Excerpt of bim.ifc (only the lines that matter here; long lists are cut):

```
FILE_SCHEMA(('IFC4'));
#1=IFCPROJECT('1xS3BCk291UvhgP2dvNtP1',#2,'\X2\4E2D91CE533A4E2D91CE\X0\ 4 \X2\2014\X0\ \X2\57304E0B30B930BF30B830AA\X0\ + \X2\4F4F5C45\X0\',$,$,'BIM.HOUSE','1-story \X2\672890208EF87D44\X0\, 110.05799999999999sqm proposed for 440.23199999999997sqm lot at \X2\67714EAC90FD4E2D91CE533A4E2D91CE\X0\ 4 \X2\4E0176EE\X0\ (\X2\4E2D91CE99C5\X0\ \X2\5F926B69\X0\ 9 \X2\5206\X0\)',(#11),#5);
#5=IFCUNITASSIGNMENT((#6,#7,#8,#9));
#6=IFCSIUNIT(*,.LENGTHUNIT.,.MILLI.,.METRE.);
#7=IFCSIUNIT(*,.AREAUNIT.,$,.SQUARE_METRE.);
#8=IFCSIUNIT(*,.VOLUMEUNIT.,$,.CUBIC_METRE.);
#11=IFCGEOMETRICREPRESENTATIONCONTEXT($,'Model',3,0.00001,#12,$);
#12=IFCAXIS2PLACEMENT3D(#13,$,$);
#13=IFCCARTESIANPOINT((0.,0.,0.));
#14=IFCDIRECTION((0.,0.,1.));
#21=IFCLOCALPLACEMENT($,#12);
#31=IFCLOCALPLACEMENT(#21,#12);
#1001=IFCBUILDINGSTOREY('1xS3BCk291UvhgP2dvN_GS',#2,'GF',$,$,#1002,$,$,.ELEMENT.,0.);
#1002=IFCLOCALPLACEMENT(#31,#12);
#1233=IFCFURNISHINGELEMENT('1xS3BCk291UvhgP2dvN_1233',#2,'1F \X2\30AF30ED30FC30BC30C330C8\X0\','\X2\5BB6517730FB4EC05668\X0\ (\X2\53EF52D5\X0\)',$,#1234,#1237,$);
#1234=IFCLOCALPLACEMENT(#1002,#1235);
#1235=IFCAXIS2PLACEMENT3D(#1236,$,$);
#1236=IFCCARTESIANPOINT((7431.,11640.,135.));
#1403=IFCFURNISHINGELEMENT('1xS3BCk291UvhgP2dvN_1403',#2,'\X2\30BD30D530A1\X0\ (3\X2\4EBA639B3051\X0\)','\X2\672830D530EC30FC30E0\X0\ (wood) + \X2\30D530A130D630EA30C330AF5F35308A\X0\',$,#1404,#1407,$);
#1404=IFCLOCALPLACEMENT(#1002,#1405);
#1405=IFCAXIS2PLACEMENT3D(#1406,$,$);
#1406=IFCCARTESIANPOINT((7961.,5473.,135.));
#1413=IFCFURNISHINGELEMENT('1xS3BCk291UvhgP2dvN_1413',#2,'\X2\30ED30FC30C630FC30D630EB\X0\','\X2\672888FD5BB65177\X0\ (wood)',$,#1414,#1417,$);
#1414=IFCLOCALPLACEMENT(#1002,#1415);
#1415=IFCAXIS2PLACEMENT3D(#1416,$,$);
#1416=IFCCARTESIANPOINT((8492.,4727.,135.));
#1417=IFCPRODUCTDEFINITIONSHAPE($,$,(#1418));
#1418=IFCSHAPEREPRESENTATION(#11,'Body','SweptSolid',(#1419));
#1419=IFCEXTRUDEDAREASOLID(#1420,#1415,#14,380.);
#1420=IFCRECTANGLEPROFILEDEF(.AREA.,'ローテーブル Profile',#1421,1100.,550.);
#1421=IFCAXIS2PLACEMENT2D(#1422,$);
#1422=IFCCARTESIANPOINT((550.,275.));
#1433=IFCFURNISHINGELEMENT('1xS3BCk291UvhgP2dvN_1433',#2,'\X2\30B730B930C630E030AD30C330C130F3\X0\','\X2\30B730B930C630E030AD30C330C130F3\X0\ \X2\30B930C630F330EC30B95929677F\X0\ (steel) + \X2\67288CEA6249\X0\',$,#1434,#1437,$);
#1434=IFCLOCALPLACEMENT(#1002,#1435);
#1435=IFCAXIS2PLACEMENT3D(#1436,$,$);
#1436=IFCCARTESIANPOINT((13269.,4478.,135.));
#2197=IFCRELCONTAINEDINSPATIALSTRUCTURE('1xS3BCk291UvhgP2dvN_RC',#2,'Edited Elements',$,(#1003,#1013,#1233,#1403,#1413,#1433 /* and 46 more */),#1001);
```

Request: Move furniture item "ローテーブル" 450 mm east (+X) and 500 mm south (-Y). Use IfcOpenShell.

```python
import ifcopenshell
import ifcopenshell.api.geometry
import ifcopenshell.util.placement
import ifcopenshell.util.unit

model = ifcopenshell.open("bim.ifc")
unit_scale = ifcopenshell.util.unit.calculate_unit_scale(model)

item = model.by_guid("1xS3BCk291UvhgP2dvN_1413")
matrix = ifcopenshell.util.placement.get_local_placement(item.ObjectPlacement)
matrix[0, 3] += 0.45 / unit_scale
matrix[1, 3] -= 0.5 / unit_scale
ifcopenshell.api.geometry.edit_object_placement(model, product=item, matrix=matrix, is_si=False)

print(ifcopenshell.util.placement.get_local_placement(item.ObjectPlacement).round(3) + 0.0)

model.write("bim_edited.ifc")
```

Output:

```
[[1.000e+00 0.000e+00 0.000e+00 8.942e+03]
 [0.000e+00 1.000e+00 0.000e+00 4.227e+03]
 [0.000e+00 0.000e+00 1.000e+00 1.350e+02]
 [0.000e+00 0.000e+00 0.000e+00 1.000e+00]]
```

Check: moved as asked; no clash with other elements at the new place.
